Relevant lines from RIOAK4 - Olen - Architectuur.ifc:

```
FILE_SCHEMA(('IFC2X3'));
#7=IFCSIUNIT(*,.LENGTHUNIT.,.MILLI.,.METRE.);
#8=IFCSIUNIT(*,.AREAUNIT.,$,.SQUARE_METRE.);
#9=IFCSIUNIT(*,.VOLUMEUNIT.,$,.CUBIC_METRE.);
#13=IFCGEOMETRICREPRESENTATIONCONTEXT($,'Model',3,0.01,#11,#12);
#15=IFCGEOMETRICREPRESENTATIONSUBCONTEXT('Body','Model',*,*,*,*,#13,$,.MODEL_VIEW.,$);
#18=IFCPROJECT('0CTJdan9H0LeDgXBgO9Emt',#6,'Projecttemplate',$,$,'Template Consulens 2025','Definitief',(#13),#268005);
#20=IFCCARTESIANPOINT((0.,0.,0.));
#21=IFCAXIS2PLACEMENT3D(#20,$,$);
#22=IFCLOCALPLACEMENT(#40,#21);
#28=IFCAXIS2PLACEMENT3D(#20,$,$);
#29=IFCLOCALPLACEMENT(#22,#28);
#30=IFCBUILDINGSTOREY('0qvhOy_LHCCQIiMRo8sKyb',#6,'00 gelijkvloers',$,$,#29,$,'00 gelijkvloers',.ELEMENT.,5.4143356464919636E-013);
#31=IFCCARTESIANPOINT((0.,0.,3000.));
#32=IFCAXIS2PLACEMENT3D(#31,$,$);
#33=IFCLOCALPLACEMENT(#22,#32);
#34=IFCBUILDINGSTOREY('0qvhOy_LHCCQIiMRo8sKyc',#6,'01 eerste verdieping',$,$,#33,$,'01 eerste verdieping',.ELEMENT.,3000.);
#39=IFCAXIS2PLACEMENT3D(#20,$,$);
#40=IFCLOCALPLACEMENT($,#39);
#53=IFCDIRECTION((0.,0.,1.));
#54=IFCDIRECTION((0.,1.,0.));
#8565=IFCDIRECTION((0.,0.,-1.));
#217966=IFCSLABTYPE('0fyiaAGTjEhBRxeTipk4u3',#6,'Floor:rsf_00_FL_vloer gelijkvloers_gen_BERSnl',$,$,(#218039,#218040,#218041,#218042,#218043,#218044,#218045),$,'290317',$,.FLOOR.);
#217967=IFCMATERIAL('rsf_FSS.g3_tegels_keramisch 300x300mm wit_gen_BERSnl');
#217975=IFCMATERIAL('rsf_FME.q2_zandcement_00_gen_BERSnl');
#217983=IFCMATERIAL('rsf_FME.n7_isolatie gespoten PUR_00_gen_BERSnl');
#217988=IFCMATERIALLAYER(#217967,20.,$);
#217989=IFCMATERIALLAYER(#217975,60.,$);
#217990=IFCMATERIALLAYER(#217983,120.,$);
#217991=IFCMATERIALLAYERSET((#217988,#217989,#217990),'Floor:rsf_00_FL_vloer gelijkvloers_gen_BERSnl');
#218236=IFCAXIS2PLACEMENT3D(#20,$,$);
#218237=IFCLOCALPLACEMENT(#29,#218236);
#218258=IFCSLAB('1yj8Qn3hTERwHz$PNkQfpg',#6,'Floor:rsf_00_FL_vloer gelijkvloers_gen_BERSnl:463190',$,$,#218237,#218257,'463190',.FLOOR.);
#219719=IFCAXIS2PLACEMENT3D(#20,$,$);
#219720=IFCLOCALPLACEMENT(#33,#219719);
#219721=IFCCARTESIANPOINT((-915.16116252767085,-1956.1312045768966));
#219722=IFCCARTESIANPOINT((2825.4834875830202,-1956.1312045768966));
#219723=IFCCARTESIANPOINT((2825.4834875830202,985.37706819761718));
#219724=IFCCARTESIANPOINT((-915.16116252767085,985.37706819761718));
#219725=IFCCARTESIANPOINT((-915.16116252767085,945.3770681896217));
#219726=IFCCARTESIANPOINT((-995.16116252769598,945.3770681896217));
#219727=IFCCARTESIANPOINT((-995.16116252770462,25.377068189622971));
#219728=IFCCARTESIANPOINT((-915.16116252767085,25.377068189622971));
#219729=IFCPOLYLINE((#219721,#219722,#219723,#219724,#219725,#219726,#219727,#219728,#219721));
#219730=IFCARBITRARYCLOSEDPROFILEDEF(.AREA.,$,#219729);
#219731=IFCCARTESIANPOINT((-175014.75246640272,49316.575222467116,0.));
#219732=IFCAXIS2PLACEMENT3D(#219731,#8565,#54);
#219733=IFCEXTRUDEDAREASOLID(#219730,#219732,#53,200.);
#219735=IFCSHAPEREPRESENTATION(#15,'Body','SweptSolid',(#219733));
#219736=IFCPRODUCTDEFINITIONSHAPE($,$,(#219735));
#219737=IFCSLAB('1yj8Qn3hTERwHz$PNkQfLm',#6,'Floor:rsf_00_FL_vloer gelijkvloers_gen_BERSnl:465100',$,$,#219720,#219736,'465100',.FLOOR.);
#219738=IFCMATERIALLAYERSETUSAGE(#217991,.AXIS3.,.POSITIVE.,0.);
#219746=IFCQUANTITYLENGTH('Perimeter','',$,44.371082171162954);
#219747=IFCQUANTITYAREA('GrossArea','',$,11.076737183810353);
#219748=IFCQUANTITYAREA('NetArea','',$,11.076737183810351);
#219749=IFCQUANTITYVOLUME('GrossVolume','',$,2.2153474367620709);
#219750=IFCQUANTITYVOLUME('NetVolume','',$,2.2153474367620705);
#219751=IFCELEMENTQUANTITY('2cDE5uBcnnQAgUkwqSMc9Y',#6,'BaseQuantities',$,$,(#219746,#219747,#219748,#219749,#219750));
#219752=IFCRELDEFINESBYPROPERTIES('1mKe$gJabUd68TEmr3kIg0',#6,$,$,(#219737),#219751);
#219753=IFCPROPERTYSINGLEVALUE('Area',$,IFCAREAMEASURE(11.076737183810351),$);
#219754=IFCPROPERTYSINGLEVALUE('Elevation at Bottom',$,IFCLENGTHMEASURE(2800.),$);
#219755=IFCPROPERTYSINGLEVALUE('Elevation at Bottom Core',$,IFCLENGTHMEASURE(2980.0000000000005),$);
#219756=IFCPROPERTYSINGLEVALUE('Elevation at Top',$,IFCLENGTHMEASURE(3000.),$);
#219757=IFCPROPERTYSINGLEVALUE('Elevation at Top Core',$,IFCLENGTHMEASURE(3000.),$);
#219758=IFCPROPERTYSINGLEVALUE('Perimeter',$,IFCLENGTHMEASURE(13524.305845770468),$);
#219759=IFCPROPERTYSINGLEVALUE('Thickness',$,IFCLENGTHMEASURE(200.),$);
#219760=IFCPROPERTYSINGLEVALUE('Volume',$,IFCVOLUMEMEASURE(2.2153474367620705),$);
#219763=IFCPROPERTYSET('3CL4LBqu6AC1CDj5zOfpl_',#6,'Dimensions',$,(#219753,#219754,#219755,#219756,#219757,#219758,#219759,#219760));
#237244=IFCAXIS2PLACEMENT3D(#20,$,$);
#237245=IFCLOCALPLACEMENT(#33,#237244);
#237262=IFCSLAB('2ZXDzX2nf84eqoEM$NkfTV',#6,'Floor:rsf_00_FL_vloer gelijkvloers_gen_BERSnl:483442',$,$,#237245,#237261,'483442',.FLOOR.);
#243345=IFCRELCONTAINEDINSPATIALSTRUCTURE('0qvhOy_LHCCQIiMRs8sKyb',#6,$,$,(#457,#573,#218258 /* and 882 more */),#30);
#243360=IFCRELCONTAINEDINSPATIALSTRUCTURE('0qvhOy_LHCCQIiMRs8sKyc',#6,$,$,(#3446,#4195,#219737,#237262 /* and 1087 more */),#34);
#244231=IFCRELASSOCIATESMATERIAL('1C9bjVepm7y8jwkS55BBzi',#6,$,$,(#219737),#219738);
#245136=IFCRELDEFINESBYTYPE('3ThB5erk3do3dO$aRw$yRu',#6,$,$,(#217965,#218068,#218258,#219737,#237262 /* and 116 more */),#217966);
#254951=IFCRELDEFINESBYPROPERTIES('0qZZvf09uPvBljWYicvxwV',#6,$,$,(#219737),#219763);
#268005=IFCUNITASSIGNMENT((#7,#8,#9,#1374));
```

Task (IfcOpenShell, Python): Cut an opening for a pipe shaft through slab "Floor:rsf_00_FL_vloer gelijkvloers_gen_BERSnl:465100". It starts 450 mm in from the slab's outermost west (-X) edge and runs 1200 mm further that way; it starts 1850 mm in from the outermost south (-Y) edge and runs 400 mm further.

```python
import numpy as np
import ifcopenshell
import ifcopenshell.api.feature
import ifcopenshell.api.geometry
import ifcopenshell.api.pset
import ifcopenshell.api.root
import ifcopenshell.geom
import ifcopenshell.util.element
import ifcopenshell.util.placement
import ifcopenshell.util.representation
import ifcopenshell.util.shape
import ifcopenshell.util.unit

model = ifcopenshell.open("RIOAK4 - Olen - Architectuur.ifc")
unit_scale = ifcopenshell.util.unit.calculate_unit_scale(model)
area_scale = ifcopenshell.util.unit.calculate_unit_scale(model, "AREAUNIT")
volume_scale = ifcopenshell.util.unit.calculate_unit_scale(model, "VOLUMEUNIT")
settings = ifcopenshell.geom.settings()


def volume(element):
    """Net volume in cubic metres, openings subtracted."""
    shape = ifcopenshell.geom.create_shape(settings, element)
    return ifcopenshell.util.shape.get_volume(shape.geometry)


slab = model.by_id(219737)
before = volume(slab)

# Extent in the slab's own axes, in metres. The edges named are its -X and -Y sides.
slab_shape = ifcopenshell.geom.create_shape(settings, slab)
vertices = ifcopenshell.util.shape.get_vertices(slab_shape.geometry)
x_min, y_min, bottom = vertices.min(axis=0)
top = vertices[:, 2].max()

opening = ifcopenshell.api.root.create_entity(model, ifc_class="IfcOpeningElement", name="Pipe shaft opening")
context = ifcopenshell.util.representation.get_context(model, "Model", "Body", "MODEL_VIEW")
width, depth = 1.2, 0.4
outline = [(0.0, 0.0), (width, 0.0), (width, depth), (0.0, depth), (0.0, 0.0)]
# Overshoot both faces by 50 mm so the cut is clean.
shape = ifcopenshell.api.geometry.add_slab_representation(
    model, context=context, depth=top - bottom + 0.1, polyline=outline
)
ifcopenshell.api.geometry.assign_representation(model, product=opening, representation=shape)

matrix = ifcopenshell.util.placement.get_local_placement(slab.ObjectPlacement)
matrix[:, 3] = matrix @ np.append(np.array([x_min + 0.45, y_min + 1.85, bottom - 0.05]) / unit_scale, 1.0)
ifcopenshell.api.geometry.edit_object_placement(model, product=opening, matrix=matrix, is_si=False)
ifcopenshell.api.feature.add_feature(model, feature=opening, element=slab)

after = volume(slab)

# Update the slab's stored quantities.
qto = model.by_id(ifcopenshell.util.element.get_pset(slab, "BaseQuantities", should_inherit=False)["id"])
ifcopenshell.api.pset.edit_qto(model, qto=qto, properties={
    "NetArea": after / (top - bottom) / area_scale,
    "NetVolume": after / volume_scale,
})
pset = model.by_id(ifcopenshell.util.element.get_pset(slab, "Dimensions", should_inherit=False)["id"])
ifcopenshell.api.pset.edit_pset(model, pset=pset, properties={
    "Area": model.create_entity("IfcAreaMeasure", after / (top - bottom) / area_scale),
    "Volume": model.create_entity("IfcVolumeMeasure", after / volume_scale),
})

print(f"slab volume {before:.3f} -> {after:.3f} m3")

model.write("RIOAK4 - Olen - Architectuur_edited.ifc")
```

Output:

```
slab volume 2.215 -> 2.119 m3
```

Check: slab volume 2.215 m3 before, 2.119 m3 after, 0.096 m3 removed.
